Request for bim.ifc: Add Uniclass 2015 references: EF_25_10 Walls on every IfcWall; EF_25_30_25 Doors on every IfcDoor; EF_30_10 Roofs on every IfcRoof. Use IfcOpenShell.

First a look at what the model holds.

```python
import ifcopenshell

model = ifcopenshell.open("bim.ifc")
print(model.schema)
print("classifications:", [c.Name for c in model.by_type("IfcClassification")])
for ifc_class in ("IfcDoor", "IfcRoof", "IfcStair", "IfcWall", "IfcWindow"):
    print(ifc_class, len(model.by_type(ifc_class)))
```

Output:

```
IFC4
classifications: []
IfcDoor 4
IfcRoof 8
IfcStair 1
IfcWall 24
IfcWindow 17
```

```python
import ifcopenshell
import ifcopenshell.api.classification

model = ifcopenshell.open("bim.ifc")

system = ifcopenshell.api.classification.add_classification(model, classification="Uniclass 2015")

codes = {
    "IfcWall": ("EF_25_10", "Walls"),
    "IfcDoor": ("EF_25_30_25", "Doors"),
    "IfcRoof": ("EF_30_10", "Roofs"),
}
for ifc_class, (code, name) in codes.items():
    products = model.by_type(ifc_class)
    ifcopenshell.api.classification.add_reference(
        model, products=products, classification=system, identification=code, name=name
    )
    print(code, len(products))

model.write("bim_updated.ifc")
```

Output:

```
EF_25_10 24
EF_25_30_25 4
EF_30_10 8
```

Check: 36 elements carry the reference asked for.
